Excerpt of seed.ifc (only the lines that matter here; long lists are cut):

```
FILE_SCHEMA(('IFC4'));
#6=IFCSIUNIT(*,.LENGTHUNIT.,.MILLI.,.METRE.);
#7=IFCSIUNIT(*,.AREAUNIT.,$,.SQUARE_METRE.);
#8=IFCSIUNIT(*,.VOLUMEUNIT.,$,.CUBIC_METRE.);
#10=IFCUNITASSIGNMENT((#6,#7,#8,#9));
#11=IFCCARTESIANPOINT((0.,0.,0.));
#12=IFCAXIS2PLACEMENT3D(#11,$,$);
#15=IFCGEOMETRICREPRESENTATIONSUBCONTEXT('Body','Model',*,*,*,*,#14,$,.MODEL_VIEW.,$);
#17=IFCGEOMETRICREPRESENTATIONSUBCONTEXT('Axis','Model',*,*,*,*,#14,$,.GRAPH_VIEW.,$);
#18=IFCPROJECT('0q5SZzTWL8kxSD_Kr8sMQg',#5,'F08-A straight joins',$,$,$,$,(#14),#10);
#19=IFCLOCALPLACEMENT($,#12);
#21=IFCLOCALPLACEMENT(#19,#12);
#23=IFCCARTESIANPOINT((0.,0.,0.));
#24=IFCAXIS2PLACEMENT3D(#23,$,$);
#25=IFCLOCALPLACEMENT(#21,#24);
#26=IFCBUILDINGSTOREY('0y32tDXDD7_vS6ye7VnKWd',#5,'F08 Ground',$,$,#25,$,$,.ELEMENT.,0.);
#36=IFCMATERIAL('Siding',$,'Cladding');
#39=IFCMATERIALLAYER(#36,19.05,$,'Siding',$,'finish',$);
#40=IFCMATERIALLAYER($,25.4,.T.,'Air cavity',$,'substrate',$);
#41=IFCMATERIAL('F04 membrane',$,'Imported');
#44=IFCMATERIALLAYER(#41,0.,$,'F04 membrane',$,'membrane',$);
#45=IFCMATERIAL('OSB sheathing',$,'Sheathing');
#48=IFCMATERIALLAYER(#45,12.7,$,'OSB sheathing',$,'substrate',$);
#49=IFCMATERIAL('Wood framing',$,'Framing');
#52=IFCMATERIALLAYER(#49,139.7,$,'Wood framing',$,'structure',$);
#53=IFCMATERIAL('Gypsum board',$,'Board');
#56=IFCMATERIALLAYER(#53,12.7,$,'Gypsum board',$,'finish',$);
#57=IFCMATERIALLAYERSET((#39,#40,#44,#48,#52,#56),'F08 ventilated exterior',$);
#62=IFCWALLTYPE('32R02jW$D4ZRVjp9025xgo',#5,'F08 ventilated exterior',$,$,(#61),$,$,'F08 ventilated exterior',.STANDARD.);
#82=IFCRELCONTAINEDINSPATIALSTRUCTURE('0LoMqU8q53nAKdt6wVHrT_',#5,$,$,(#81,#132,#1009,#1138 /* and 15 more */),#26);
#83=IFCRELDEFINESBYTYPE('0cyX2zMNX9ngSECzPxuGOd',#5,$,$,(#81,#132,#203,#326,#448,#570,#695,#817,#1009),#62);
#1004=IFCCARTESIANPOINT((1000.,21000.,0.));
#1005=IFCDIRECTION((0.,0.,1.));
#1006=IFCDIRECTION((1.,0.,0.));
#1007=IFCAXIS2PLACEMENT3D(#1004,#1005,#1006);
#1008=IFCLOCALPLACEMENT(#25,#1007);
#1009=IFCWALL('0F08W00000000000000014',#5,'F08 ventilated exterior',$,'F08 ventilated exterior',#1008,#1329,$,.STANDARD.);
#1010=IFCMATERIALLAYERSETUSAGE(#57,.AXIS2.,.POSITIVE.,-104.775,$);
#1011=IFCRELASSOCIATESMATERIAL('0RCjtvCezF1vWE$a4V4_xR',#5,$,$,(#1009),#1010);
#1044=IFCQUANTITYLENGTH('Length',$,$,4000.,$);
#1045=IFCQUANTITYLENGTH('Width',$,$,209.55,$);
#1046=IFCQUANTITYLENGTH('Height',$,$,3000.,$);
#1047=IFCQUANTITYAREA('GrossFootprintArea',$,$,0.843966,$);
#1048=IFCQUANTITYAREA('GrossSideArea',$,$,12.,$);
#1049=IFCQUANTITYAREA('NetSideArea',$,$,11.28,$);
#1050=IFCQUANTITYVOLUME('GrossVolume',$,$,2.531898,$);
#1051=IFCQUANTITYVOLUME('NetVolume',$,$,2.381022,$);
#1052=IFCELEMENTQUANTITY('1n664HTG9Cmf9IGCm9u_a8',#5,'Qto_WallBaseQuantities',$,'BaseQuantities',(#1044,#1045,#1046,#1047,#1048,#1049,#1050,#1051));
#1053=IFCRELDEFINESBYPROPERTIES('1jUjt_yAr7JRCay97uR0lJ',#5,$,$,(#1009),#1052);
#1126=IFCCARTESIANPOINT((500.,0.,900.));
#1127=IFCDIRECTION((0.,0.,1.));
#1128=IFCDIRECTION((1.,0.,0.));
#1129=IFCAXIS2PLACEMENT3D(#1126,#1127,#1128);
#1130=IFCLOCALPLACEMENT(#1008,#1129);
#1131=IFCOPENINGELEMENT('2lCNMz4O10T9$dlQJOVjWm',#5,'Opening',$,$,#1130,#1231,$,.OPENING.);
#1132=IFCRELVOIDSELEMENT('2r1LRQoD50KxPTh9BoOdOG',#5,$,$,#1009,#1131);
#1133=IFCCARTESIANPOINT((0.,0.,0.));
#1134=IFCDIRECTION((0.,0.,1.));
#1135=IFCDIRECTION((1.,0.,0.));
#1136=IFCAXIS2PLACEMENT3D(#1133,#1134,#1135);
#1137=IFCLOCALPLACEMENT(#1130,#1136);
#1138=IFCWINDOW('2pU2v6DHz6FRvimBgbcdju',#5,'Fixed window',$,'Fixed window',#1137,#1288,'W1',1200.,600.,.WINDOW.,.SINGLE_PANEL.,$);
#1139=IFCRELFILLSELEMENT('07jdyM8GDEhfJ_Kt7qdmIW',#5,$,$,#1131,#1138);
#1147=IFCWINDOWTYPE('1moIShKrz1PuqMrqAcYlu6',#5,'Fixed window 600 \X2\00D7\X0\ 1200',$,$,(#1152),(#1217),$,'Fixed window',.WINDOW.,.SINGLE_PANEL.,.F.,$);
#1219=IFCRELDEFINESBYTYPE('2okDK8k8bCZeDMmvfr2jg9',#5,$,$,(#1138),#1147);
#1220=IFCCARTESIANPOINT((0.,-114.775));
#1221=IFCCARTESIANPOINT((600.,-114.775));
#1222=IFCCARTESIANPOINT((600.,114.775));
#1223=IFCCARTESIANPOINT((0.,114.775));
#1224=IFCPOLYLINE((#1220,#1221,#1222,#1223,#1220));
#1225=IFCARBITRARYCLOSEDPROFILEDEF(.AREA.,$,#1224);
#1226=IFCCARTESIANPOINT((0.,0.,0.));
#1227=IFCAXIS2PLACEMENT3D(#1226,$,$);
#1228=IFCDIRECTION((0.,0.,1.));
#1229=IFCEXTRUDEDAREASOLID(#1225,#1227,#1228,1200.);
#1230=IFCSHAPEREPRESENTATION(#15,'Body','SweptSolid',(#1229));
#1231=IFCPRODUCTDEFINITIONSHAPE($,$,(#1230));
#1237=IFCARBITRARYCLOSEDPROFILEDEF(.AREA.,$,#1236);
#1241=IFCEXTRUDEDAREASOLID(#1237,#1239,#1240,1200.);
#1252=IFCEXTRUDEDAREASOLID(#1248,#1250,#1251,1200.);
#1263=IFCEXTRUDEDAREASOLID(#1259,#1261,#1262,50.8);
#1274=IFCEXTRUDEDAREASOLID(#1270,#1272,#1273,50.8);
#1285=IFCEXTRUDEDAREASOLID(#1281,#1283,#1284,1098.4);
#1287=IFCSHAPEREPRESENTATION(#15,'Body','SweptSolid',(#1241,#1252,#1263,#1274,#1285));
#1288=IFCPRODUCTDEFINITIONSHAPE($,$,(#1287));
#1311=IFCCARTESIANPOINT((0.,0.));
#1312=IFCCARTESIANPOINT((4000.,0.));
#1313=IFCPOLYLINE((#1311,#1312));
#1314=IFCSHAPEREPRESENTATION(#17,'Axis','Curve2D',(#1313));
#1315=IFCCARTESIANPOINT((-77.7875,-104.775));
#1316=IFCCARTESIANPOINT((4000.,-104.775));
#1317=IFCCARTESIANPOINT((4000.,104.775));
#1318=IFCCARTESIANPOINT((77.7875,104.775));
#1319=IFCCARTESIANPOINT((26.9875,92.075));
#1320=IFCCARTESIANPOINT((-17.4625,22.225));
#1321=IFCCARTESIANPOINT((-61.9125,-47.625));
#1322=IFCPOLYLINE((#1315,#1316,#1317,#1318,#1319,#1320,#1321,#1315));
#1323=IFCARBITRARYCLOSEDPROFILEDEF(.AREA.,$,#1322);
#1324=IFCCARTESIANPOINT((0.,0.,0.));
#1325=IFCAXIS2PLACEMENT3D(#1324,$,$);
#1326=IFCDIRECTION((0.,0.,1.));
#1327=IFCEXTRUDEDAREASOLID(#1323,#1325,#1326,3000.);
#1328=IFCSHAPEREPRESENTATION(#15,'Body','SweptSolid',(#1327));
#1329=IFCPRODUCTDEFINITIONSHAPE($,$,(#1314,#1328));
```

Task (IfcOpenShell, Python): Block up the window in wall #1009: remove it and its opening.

```python
import ifcopenshell
import ifcopenshell.api.feature
import ifcopenshell.api.pset
import ifcopenshell.api.root
import ifcopenshell.geom
import ifcopenshell.util.element
import ifcopenshell.util.shape
import ifcopenshell.util.unit

model = ifcopenshell.open("seed.ifc")
area_scale = ifcopenshell.util.unit.calculate_unit_scale(model, "AREAUNIT")
volume_scale = ifcopenshell.util.unit.calculate_unit_scale(model, "VOLUMEUNIT")
settings = ifcopenshell.geom.settings()


def volume(element):
    """Net volume in cubic metres, openings subtracted."""
    shape = ifcopenshell.geom.create_shape(settings, element)
    return ifcopenshell.util.shape.get_volume(shape.geometry)


window = model.by_guid("2pU2v6DHz6FRvimBgbcdju")
opening = window.FillsVoids[0].RelatingOpeningElement
wall = opening.VoidsElements[0].RelatingBuildingElement
before = volume(wall)

ifcopenshell.api.root.remove_product(model, product=window)
ifcopenshell.api.feature.remove_feature(model, feature=opening)

after = volume(wall)
thickness = 0.2096  # wall thickness in metres

# Update the wall's stored quantities.
qto = model.by_id(ifcopenshell.util.element.get_pset(wall, "Qto_WallBaseQuantities", should_inherit=False)["id"])
ifcopenshell.api.pset.edit_qto(model, qto=qto, properties={
    "NetSideArea": after / thickness / area_scale,
    "NetVolume": after / volume_scale,
})

print(f"wall volume {before:.3f} -> {after:.3f} m3")

model.write("seed_rev.ifc")
```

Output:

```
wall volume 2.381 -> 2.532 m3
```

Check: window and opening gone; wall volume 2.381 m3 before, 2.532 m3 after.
